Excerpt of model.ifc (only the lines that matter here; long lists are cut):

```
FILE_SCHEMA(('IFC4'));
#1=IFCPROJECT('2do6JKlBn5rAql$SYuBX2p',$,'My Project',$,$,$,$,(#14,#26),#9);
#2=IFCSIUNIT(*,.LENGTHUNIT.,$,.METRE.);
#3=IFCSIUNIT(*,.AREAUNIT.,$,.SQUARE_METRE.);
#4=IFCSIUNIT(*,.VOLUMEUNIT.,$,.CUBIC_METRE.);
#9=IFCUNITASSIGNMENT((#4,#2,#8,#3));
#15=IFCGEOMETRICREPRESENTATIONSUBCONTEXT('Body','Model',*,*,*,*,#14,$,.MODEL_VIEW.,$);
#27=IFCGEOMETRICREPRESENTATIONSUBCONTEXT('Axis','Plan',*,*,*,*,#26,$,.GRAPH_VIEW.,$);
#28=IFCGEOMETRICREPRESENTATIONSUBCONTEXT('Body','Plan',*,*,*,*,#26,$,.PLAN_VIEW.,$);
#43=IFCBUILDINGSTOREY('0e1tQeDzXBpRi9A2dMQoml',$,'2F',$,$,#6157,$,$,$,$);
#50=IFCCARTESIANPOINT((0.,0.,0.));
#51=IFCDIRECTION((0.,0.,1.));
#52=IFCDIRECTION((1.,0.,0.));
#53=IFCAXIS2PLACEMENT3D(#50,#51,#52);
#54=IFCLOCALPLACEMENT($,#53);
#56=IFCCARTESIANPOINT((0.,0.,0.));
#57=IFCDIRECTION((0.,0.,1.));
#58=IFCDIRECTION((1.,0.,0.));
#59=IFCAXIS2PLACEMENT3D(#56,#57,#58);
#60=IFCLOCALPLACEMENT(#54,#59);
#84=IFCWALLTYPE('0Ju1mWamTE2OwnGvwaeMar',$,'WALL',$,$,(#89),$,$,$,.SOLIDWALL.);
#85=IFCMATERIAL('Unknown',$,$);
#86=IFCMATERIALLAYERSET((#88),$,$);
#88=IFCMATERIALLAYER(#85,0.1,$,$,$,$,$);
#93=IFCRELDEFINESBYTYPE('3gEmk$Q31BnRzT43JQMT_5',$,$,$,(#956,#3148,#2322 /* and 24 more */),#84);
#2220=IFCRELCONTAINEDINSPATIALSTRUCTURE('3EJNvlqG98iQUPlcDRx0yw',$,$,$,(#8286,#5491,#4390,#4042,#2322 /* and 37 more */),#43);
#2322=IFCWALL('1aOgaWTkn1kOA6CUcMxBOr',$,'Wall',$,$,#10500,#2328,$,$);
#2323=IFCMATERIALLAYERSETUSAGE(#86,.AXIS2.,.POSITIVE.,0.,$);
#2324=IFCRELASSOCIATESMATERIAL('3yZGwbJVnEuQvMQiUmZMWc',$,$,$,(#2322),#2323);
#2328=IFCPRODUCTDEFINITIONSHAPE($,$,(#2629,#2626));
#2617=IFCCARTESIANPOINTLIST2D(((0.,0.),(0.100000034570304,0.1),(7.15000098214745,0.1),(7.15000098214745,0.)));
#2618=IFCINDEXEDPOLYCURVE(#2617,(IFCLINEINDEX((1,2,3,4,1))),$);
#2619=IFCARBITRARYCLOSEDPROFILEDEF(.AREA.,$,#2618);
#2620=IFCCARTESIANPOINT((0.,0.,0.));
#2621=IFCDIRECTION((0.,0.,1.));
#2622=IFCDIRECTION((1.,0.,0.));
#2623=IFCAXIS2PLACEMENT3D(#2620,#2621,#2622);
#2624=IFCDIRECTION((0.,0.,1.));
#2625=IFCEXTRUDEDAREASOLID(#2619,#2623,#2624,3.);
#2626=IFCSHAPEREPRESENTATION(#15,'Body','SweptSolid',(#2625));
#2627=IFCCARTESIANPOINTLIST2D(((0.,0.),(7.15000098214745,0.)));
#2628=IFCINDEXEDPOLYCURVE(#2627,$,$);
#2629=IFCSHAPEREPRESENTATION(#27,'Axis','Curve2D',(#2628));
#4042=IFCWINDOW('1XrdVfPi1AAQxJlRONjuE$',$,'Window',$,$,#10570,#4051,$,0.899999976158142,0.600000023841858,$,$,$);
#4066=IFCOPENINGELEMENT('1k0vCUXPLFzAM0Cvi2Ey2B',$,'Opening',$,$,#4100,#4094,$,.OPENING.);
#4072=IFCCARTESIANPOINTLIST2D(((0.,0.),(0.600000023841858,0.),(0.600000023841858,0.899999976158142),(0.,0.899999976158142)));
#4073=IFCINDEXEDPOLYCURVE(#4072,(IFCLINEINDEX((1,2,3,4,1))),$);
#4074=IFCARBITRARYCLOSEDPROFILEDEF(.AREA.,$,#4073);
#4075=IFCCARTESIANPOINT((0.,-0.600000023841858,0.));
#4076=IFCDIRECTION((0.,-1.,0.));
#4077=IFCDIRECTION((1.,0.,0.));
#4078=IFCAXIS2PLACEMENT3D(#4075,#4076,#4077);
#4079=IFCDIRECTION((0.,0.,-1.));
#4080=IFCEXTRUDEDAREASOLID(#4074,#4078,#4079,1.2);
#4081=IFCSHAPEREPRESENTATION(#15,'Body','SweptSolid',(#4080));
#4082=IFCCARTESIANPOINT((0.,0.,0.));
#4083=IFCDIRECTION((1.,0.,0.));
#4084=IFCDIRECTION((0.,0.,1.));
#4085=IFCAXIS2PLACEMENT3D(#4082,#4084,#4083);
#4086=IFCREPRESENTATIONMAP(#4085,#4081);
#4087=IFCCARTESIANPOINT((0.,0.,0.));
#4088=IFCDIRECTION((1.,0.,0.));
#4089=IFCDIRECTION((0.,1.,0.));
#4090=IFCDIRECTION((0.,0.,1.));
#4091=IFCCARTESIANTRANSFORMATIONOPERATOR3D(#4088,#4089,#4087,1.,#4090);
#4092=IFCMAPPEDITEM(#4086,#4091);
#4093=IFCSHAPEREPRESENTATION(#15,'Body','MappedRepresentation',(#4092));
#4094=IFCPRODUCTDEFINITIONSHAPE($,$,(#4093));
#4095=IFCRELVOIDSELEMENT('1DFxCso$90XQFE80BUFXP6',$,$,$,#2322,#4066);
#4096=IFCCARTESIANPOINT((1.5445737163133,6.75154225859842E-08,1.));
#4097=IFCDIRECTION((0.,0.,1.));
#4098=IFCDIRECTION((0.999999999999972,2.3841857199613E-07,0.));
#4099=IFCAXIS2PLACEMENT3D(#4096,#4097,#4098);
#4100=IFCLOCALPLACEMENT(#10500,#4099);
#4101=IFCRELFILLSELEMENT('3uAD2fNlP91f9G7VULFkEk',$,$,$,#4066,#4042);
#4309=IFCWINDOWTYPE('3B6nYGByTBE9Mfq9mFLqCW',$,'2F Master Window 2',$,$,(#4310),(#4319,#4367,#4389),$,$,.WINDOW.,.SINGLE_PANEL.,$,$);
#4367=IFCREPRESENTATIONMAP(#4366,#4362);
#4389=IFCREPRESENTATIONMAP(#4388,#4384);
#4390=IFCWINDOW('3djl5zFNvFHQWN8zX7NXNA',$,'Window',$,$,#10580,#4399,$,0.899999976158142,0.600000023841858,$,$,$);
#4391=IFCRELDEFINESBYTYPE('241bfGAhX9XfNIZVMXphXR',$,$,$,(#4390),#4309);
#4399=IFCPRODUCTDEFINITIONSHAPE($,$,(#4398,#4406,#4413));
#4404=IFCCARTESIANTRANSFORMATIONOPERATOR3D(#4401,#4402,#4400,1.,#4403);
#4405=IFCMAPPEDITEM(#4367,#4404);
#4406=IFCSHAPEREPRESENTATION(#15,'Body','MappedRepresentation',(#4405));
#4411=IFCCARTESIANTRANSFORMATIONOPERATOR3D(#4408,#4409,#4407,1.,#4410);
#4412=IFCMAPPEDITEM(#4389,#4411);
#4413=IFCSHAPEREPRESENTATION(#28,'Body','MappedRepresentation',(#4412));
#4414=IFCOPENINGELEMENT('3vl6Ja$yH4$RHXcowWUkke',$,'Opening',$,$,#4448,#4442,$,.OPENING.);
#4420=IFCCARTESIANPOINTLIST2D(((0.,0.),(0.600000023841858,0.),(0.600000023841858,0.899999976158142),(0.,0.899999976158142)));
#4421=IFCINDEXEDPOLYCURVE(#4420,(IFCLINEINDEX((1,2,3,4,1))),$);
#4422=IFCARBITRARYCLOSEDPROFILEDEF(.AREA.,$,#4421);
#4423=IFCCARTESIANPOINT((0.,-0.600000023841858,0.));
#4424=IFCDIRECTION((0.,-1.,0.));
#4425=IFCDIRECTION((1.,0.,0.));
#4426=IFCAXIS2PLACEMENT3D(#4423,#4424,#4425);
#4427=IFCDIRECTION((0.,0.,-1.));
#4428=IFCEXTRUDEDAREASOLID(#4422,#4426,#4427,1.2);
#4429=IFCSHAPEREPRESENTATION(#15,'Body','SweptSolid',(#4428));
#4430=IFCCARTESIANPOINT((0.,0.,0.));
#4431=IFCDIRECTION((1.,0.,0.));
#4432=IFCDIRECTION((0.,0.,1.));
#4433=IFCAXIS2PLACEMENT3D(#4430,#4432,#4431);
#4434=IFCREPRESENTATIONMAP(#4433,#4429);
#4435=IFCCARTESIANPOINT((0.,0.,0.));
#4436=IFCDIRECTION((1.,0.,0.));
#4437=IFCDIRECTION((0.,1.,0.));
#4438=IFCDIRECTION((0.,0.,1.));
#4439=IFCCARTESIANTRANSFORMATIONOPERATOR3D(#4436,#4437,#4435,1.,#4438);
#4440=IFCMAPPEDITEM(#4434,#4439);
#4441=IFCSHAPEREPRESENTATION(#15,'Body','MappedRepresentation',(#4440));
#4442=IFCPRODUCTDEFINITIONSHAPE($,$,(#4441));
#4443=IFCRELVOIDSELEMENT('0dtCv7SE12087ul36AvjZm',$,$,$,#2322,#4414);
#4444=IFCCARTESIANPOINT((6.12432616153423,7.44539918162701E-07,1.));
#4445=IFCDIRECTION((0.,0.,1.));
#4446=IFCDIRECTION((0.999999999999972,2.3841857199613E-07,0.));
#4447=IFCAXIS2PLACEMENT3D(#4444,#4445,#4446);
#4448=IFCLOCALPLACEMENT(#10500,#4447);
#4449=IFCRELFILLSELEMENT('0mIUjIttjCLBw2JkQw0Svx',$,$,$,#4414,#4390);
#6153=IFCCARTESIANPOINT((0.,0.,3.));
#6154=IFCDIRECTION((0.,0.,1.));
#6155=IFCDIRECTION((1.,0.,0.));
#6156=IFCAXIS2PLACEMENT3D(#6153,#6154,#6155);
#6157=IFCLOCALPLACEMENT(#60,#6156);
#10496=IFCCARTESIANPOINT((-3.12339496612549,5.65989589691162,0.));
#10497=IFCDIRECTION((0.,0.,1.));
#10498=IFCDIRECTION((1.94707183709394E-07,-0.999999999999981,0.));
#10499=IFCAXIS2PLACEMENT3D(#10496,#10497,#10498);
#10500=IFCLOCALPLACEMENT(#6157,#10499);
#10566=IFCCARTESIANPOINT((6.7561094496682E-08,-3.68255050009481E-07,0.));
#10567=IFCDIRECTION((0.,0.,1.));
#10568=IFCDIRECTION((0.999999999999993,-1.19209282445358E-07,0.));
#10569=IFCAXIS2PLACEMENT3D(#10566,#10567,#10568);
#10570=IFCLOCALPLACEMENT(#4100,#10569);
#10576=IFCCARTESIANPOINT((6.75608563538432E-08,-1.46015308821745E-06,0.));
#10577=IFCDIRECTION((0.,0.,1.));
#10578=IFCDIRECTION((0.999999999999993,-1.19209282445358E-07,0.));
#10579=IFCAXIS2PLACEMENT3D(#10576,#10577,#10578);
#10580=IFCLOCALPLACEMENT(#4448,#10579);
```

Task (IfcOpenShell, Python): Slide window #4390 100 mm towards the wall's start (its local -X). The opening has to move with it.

```python
import ifcopenshell
import ifcopenshell.api.geometry
import ifcopenshell.util.placement

model = ifcopenshell.open("model.ifc")

window = model.by_guid("3djl5zFNvFHQWN8zX7NXNA")
opening = window.FillsVoids[0].RelatingOpeningElement
wall = opening.VoidsElements[0].RelatingBuildingElement

wall_matrix = ifcopenshell.util.placement.get_local_placement(wall.ObjectPlacement)
shift = wall_matrix[:3, 0] * -0.1
before = ifcopenshell.util.placement.get_local_placement(window.ObjectPlacement)[:3, 3].copy()

# The window is placed relative to its opening, so it follows when the opening moves.
matrix = ifcopenshell.util.placement.get_local_placement(opening.ObjectPlacement)
matrix[:3, 3] += shift
ifcopenshell.api.geometry.edit_object_placement(
    model, product=opening, matrix=matrix, is_si=False, should_transform_children=True
)

after = ifcopenshell.util.placement.get_local_placement(window.ObjectPlacement)[:3, 3]
print("window moved by", (after - before).round(3) + 0.0)

model.write("model_rev.ifc")
```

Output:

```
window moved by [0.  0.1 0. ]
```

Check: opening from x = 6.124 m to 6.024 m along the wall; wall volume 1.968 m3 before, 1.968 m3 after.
